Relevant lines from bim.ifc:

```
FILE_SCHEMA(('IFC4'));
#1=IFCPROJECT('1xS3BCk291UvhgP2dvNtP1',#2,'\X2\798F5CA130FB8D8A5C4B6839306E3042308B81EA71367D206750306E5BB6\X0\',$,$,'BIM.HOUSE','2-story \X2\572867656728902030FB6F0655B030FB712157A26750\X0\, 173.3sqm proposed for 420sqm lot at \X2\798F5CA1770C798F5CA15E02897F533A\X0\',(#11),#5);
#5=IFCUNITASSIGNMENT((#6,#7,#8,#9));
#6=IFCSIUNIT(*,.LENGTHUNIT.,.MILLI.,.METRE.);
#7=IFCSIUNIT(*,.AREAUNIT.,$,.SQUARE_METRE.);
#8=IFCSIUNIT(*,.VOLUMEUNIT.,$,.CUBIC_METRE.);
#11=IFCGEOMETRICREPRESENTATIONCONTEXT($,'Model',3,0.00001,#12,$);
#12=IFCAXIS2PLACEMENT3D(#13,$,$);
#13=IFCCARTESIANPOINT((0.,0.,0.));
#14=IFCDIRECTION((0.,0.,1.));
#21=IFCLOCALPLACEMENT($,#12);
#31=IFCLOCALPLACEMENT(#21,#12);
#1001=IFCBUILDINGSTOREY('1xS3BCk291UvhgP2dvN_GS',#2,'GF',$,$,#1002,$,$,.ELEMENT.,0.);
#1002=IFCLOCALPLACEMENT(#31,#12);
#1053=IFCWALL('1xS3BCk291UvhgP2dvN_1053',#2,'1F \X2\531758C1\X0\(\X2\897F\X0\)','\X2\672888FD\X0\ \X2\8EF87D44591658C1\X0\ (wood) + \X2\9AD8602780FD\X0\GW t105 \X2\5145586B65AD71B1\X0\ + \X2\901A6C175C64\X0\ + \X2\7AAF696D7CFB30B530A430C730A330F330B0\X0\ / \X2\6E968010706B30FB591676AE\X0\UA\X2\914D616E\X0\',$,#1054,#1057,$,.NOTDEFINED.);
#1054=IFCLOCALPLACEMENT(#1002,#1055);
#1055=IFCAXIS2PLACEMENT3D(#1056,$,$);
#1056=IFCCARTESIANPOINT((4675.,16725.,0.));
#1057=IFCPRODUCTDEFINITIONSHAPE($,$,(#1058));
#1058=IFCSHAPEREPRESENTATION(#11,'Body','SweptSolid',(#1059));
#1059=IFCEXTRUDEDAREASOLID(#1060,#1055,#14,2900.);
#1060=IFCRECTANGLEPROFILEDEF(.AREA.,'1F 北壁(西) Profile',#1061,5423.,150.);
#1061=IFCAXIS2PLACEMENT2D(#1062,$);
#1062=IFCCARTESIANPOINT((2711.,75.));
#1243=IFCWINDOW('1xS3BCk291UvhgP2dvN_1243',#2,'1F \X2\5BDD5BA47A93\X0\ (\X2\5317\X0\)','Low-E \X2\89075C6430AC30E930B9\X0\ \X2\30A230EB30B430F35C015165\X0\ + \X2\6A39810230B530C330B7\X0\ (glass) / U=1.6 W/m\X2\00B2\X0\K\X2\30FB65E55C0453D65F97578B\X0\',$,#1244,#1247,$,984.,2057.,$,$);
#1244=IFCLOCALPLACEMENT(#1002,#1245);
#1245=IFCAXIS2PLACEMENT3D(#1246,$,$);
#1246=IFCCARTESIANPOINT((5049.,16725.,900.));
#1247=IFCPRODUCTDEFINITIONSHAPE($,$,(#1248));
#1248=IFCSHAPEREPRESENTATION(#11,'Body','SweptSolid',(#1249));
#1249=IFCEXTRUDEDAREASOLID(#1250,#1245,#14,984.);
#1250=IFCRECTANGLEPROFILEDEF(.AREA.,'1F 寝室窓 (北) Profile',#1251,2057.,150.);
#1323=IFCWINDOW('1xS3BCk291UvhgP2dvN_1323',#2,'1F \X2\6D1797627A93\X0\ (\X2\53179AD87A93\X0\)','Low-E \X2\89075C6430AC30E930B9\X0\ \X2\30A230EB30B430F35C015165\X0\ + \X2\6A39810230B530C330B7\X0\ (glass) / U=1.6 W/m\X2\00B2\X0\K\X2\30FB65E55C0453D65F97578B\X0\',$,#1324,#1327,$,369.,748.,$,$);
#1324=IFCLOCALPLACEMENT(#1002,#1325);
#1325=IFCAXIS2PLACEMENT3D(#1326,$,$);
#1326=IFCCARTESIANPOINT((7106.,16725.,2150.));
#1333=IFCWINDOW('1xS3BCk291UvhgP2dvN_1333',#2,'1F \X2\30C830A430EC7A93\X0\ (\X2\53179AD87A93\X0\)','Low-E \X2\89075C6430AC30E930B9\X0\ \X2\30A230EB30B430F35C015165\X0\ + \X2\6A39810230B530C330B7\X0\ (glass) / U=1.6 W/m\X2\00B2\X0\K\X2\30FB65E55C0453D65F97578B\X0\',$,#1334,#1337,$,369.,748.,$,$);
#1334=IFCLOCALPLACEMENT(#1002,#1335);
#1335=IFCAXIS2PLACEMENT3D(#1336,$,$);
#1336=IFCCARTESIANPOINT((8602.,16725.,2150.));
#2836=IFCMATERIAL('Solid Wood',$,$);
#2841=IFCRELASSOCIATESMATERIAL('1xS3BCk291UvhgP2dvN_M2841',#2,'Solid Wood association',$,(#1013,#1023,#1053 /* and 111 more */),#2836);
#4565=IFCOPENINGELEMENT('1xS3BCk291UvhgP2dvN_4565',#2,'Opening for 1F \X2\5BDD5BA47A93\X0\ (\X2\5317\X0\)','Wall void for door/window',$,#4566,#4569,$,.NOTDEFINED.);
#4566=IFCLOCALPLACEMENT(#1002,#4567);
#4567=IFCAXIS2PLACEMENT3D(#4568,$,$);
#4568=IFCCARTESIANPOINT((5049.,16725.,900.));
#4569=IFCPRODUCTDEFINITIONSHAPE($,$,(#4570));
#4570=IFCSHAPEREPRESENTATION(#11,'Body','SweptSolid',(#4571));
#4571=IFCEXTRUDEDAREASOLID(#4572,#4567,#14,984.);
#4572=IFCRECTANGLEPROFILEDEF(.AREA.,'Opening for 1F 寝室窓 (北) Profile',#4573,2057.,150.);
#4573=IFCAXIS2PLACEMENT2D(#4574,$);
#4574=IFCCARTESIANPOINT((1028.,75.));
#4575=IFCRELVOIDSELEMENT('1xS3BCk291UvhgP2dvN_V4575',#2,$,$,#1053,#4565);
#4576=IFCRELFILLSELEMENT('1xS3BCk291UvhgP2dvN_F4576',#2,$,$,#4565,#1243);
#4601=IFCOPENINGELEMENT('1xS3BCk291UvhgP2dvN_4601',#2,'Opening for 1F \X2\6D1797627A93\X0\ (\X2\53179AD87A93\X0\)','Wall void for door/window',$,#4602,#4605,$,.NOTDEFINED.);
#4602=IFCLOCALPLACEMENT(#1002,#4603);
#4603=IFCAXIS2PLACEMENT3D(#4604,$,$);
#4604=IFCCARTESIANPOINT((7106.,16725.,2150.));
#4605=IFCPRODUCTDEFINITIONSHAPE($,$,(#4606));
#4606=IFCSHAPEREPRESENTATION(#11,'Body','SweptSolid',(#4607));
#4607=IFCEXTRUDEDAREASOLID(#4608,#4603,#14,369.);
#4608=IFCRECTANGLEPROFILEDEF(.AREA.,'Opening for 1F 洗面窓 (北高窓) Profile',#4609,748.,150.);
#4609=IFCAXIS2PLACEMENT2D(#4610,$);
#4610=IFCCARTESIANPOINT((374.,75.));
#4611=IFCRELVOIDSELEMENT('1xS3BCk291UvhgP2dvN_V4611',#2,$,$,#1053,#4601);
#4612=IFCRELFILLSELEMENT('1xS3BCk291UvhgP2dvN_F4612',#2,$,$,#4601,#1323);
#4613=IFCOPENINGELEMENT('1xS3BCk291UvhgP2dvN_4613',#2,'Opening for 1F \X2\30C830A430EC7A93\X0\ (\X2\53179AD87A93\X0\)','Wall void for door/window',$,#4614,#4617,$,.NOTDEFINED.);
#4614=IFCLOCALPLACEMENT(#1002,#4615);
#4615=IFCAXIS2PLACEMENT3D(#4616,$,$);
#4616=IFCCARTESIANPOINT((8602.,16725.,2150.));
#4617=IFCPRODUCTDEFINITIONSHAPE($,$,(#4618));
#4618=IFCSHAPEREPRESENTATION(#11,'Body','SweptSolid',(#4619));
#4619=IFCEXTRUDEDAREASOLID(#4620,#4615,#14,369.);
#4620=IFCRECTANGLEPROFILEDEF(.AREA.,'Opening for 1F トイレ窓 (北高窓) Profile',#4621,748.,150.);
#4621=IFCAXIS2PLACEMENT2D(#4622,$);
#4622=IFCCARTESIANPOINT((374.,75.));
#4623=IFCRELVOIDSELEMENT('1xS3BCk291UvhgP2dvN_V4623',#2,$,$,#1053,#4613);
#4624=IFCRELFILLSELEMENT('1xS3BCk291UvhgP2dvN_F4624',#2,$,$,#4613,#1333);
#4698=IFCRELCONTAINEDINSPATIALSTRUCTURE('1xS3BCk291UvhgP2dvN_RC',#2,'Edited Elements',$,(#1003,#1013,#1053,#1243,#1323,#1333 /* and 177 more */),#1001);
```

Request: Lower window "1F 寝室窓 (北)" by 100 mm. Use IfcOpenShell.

```python
import numpy as np
import ifcopenshell
import ifcopenshell.api.geometry
import ifcopenshell.util.placement
import ifcopenshell.util.unit

model = ifcopenshell.open("bim.ifc")
unit_scale = ifcopenshell.util.unit.calculate_unit_scale(model)

window = model.by_guid("1xS3BCk291UvhgP2dvN_1243")
opening = window.FillsVoids[0].RelatingOpeningElement
dz = -0.1 / unit_scale

shift = np.array([0.0, 0.0, dz])
# The window is not placed relative to its opening, so move both.
for product in (opening, window):
    matrix = ifcopenshell.util.placement.get_local_placement(product.ObjectPlacement)
    matrix[:3, 3] += shift
    ifcopenshell.api.geometry.edit_object_placement(model, product=product, matrix=matrix, is_si=False)

print(f"moved by {dz * unit_scale:+.3f} m")

model.write("bim_edited.ifc")
```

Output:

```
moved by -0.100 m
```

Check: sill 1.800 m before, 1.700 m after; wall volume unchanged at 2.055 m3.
